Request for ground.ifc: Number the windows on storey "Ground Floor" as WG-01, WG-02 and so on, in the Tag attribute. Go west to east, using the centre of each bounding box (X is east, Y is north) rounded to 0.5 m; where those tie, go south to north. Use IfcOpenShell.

First a look at what the model holds.

```python
import ifcopenshell
import ifcopenshell.util.element
import ifcopenshell.util.placement

model = ifcopenshell.open("ground.ifc")
print(model.schema)
storey = next(s for s in model.by_type("IfcBuildingStorey") if s.Name == "Ground Floor")
windows = [e for e in ifcopenshell.util.element.get_decomposition(storey) if e.is_a("IfcWindow")]
for e in sorted(windows, key=lambda e: e.id()):
    origin = ifcopenshell.util.placement.get_local_placement(e.ObjectPlacement)[:3, 3]
    print(e.id(), e.Tag, e.Name, origin.round(2) + 0.0, sep=" | ")
```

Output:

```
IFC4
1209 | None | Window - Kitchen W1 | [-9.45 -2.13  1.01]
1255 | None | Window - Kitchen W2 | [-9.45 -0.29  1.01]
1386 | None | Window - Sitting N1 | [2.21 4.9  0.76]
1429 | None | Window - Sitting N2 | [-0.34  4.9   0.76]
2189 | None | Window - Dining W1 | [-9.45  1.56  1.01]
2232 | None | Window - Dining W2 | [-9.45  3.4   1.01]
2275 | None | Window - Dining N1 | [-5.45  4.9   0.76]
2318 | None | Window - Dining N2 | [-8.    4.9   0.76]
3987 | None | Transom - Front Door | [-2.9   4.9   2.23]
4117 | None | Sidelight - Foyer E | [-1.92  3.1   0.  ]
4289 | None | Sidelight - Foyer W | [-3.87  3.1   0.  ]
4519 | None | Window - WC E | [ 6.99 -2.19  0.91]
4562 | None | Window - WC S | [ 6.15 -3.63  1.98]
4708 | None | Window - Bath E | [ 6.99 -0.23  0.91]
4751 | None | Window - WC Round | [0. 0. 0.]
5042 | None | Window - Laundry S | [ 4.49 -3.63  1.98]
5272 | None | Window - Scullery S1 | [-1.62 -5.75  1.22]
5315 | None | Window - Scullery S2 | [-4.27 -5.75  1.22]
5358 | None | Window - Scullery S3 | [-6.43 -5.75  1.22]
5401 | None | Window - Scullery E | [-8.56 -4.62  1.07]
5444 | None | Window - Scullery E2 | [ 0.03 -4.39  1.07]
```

```python
import ifcopenshell
import ifcopenshell.geom
import ifcopenshell.util.element
import ifcopenshell.util.shape

model = ifcopenshell.open("ground.ifc")
settings = ifcopenshell.geom.settings()
settings.set("use-world-coords", True)


def centre(element):
    shape = ifcopenshell.geom.create_shape(settings, element)
    return ifcopenshell.util.shape.get_bbox_centroid(shape.geometry)


storey = next(s for s in model.by_type("IfcBuildingStorey") if s.Name == "Ground Floor")
windows = [e for e in ifcopenshell.util.element.get_decomposition(storey) if e.is_a("IfcWindow")]

# Insertion points can sit at a corner or the storey origin, so sort by the geometry (in metres).
centres = {e: centre(e) for e in windows}
windows.sort(key=lambda e: (round(centres[e][0] / 0.5), centres[e][1]))

for i, e in enumerate(windows, start=1):
    number = f"WG-{i:02d}"
    e.Tag = number
    print(e.id(), number)

model.write("ground-out.ifc")
```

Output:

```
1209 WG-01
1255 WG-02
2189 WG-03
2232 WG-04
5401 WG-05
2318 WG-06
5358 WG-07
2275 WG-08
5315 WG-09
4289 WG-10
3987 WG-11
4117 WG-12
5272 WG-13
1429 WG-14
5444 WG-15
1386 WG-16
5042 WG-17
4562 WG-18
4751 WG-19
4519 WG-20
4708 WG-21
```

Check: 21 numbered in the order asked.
